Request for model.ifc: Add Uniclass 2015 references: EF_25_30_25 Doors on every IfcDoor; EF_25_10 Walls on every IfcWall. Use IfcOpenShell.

First a look at what the model holds.

```python
import ifcopenshell

model = ifcopenshell.open("model.ifc")
print(model.schema)
print("classifications:", [c.Name for c in model.by_type("IfcClassification")])
for ifc_class in ("IfcDoor", "IfcRoof", "IfcStair", "IfcWall", "IfcWindow"):
    print(ifc_class, len(model.by_type(ifc_class)))
```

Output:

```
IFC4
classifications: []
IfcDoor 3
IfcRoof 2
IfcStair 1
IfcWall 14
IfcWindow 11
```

```python
import ifcopenshell
import ifcopenshell.api.classification

model = ifcopenshell.open("model.ifc")

system = ifcopenshell.api.classification.add_classification(model, classification="Uniclass 2015")

codes = {
    "IfcDoor": ("EF_25_30_25", "Doors"),
    "IfcWall": ("EF_25_10", "Walls"),
}
for ifc_class, (code, name) in codes.items():
    products = model.by_type(ifc_class)
    ifcopenshell.api.classification.add_reference(
        model, products=products, classification=system, identification=code, name=name
    )
    print(code, len(products))

model.write("model_edited.ifc")
```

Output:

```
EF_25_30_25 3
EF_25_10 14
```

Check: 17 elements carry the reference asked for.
